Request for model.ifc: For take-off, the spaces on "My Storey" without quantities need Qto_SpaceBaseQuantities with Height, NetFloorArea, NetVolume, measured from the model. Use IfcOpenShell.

First a look at what the model holds.

```python
import ifcopenshell
import ifcopenshell.util.element
import ifcopenshell.util.unit

model = ifcopenshell.open("model.ifc")
print(model.schema)
for unit_type in ("LENGTHUNIT", "AREAUNIT", "VOLUMEUNIT"):
    print(unit_type, ifcopenshell.util.unit.calculate_unit_scale(model, unit_type))
storey = next(s for s in model.by_type("IfcBuildingStorey") if s.Name == "My Storey")
spaces = [e for e in ifcopenshell.util.element.get_decomposition(storey) if e.is_a("IfcSpace")]
for e in sorted(spaces, key=lambda e: e.id()):
    print(e.id(), e.is_a(), e.Name, list(ifcopenshell.util.element.get_psets(e, qtos_only=True)), sep=" | ")
```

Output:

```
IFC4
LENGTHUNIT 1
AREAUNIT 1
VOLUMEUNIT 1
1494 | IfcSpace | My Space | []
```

```python
import ifcopenshell
import ifcopenshell.api.pset
import ifcopenshell.geom
import ifcopenshell.util.element
import ifcopenshell.util.shape
import ifcopenshell.util.unit

model = ifcopenshell.open("model.ifc")
unit_scale = ifcopenshell.util.unit.calculate_unit_scale(model)
area_scale = ifcopenshell.util.unit.calculate_unit_scale(model, "AREAUNIT")
volume_scale = ifcopenshell.util.unit.calculate_unit_scale(model, "VOLUMEUNIT")
settings = ifcopenshell.geom.settings()

storey = next(s for s in model.by_type("IfcBuildingStorey") if s.Name == "My Storey")
spaces = [e for e in ifcopenshell.util.element.get_decomposition(storey) if e.is_a("IfcSpace")]

for e in sorted(spaces, key=lambda e: e.id()):
    if ifcopenshell.util.element.get_psets(e, qtos_only=True, should_inherit=False):
        continue
    # Geometry comes back in metres, in the element's own axes.
    shape = ifcopenshell.geom.create_shape(settings, e)
    values = {
        "Height": ifcopenshell.util.shape.get_z(shape.geometry) / unit_scale,
        "NetFloorArea": ifcopenshell.util.shape.get_footprint_area(shape.geometry) / area_scale,
        "NetVolume": ifcopenshell.util.shape.get_volume(shape.geometry) / volume_scale,
    }
    qto = ifcopenshell.api.pset.add_qto(model, product=e, name="Qto_SpaceBaseQuantities")
    ifcopenshell.api.pset.edit_qto(model, qto=qto, properties=values)
    print(e.id(), {k: round(v, 3) for k, v in values.items()})

model.write("model_updated.ifc")
```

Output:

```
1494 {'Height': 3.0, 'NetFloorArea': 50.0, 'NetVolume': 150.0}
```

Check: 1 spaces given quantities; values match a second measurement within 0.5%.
